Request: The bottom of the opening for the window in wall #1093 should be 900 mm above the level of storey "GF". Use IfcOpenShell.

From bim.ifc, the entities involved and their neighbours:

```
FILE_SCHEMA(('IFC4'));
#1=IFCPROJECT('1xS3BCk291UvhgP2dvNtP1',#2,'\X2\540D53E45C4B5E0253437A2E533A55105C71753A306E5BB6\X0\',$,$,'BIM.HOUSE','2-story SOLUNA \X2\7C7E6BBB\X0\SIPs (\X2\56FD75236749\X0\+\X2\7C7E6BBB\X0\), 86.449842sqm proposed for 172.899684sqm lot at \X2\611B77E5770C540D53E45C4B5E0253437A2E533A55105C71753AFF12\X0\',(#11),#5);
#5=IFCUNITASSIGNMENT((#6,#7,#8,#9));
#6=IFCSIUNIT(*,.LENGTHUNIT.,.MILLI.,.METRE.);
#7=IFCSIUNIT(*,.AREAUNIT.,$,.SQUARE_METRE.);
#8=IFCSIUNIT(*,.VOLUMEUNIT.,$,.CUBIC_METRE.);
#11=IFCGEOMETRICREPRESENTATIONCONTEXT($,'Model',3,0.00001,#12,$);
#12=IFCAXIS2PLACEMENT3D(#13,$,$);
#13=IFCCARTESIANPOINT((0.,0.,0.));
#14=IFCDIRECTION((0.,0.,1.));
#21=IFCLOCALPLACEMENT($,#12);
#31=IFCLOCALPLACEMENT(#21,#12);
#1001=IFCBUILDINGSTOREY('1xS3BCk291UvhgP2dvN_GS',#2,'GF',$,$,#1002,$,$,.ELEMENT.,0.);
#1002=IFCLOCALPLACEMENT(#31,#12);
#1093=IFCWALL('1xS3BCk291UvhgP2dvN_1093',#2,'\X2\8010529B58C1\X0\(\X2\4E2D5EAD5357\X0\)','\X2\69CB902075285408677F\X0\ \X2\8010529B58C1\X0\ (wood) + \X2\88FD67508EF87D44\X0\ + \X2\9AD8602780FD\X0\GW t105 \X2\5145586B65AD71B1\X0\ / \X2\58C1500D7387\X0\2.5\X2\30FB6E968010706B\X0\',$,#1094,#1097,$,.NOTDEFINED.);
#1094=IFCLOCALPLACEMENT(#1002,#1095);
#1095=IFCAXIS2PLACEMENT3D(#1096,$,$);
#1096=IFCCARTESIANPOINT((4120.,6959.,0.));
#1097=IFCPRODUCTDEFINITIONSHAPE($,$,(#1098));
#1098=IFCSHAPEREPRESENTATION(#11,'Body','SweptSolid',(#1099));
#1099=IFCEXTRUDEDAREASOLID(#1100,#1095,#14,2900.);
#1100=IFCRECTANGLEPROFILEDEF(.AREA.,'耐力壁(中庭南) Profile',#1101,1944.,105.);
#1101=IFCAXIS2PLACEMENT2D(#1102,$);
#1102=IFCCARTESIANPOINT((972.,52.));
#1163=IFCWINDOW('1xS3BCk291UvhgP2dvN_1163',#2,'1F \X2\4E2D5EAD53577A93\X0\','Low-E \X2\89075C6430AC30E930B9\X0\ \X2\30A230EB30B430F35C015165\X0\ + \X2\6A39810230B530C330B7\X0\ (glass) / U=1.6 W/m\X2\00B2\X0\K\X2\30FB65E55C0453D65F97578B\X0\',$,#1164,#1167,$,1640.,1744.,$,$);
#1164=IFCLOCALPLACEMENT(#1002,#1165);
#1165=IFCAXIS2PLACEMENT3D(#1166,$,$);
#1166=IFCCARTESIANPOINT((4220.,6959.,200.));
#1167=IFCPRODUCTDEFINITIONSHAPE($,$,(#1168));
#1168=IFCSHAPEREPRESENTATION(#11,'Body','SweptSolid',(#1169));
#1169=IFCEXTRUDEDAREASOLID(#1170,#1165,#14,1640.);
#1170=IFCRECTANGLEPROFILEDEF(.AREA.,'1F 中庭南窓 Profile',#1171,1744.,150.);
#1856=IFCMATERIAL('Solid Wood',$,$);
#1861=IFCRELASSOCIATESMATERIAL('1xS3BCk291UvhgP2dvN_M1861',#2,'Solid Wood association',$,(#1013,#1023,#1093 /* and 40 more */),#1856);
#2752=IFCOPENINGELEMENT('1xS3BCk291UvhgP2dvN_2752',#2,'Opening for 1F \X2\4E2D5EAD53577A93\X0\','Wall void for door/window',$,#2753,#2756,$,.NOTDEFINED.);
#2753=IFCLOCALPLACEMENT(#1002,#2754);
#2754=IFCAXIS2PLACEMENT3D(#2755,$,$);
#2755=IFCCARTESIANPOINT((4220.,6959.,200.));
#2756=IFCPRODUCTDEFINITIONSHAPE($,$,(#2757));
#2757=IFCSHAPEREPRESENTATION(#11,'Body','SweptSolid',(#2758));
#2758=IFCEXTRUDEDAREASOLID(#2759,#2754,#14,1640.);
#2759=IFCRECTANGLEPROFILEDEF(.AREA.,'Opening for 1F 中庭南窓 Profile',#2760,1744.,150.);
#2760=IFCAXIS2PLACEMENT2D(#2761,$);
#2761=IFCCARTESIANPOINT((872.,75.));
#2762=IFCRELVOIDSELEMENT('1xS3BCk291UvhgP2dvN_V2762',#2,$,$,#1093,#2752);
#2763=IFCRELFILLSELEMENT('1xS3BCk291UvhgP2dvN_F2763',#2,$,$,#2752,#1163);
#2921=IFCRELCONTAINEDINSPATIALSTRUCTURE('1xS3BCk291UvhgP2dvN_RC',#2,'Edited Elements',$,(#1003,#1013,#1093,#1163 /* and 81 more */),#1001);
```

```python
import numpy as np
import ifcopenshell
import ifcopenshell.api.geometry
import ifcopenshell.geom
import ifcopenshell.util.element
import ifcopenshell.util.placement
import ifcopenshell.util.shape
import ifcopenshell.util.unit

model = ifcopenshell.open("bim.ifc")
unit_scale = ifcopenshell.util.unit.calculate_unit_scale(model)

window = model.by_guid("1xS3BCk291UvhgP2dvN_1163")
opening = window.FillsVoids[0].RelatingOpeningElement
storey = ifcopenshell.util.element.get_container(window, ifc_class="IfcBuildingStorey")
level = ifcopenshell.util.placement.get_local_placement(storey.ObjectPlacement)[2, 3]

# The opening's origin need not be at the sill, so measure its lowest point.
shape = ifcopenshell.geom.create_shape(ifcopenshell.geom.settings(), opening)
bottom = ifcopenshell.util.shape.get_shape_bottom_elevation(shape, shape.geometry) / unit_scale
dz = level + 0.9 / unit_scale - bottom

shift = np.array([0.0, 0.0, dz])
# The window is not placed relative to its opening, so move both.
for product in (opening, window):
    matrix = ifcopenshell.util.placement.get_local_placement(product.ObjectPlacement)
    matrix[:3, 3] += shift
    ifcopenshell.api.geometry.edit_object_placement(model, product=product, matrix=matrix, is_si=False)

print(f"moved by {dz * unit_scale:+.3f} m")

model.write("bim_edited.ifc")
```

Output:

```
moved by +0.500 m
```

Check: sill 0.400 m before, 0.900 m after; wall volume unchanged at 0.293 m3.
